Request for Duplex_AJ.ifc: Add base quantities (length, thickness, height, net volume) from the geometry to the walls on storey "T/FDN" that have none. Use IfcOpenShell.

First a look at what the model holds.

```python
import ifcopenshell
import ifcopenshell.util.element
import ifcopenshell.util.unit

model = ifcopenshell.open("Duplex_AJ.ifc")
print(model.schema)
for unit_type in ("LENGTHUNIT", "AREAUNIT", "VOLUMEUNIT"):
    print(unit_type, ifcopenshell.util.unit.calculate_unit_scale(model, unit_type))
storey = next(s for s in model.by_type("IfcBuildingStorey") if s.Name == "T/FDN")
walls = [e for e in ifcopenshell.util.element.get_decomposition(storey) if e.is_a("IfcWall")]
for e in sorted(walls, key=lambda e: e.id()):
    print(e.id(), e.is_a(), e.Name, list(ifcopenshell.util.element.get_psets(e, qtos_only=True)), sep=" | ")
```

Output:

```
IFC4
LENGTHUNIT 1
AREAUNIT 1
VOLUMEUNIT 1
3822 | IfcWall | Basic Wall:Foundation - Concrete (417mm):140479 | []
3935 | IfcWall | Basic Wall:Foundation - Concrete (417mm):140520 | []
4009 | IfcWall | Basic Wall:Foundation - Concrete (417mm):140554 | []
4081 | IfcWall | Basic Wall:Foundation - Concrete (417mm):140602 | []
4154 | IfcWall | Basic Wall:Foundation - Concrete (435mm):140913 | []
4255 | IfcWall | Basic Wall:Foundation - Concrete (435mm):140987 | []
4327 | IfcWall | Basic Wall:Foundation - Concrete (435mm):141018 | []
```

```python
import ifcopenshell
import ifcopenshell.api.pset
import ifcopenshell.geom
import ifcopenshell.util.element
import ifcopenshell.util.shape
import ifcopenshell.util.unit

model = ifcopenshell.open("Duplex_AJ.ifc")
unit_scale = ifcopenshell.util.unit.calculate_unit_scale(model)
volume_scale = ifcopenshell.util.unit.calculate_unit_scale(model, "VOLUMEUNIT")
settings = ifcopenshell.geom.settings()

storey = next(s for s in model.by_type("IfcBuildingStorey") if s.Name == "T/FDN")
walls = [e for e in ifcopenshell.util.element.get_decomposition(storey) if e.is_a("IfcWall")]

for e in sorted(walls, key=lambda e: e.id()):
    if ifcopenshell.util.element.get_psets(e, qtos_only=True, should_inherit=False):
        continue
    # Geometry comes back in metres, in the element's own axes.
    shape = ifcopenshell.geom.create_shape(settings, e)
    values = {
        "Length": ifcopenshell.util.shape.get_x(shape.geometry) / unit_scale,
        "Width": ifcopenshell.util.shape.get_y(shape.geometry) / unit_scale,
        "Height": ifcopenshell.util.shape.get_z(shape.geometry) / unit_scale,
        "NetVolume": ifcopenshell.util.shape.get_volume(shape.geometry) / volume_scale,
    }
    qto = ifcopenshell.api.pset.add_qto(model, product=e, name="Qto_WallBaseQuantities")
    ifcopenshell.api.pset.edit_qto(model, qto=qto, properties=values)
    print(e.id(), {k: round(v, 3) for k, v in values.items()})

model.write("Duplex_AJ_v2.ifc")
```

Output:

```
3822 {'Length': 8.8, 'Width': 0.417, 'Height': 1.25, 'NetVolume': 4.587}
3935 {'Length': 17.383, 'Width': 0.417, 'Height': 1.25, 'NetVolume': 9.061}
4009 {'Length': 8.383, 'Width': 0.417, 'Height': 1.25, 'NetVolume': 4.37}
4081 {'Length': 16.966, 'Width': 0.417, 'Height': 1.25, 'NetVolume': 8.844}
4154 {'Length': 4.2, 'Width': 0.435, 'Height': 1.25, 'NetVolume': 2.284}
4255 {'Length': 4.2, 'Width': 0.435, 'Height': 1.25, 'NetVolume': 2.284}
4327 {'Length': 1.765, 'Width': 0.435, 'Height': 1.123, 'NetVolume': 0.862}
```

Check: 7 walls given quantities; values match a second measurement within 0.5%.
